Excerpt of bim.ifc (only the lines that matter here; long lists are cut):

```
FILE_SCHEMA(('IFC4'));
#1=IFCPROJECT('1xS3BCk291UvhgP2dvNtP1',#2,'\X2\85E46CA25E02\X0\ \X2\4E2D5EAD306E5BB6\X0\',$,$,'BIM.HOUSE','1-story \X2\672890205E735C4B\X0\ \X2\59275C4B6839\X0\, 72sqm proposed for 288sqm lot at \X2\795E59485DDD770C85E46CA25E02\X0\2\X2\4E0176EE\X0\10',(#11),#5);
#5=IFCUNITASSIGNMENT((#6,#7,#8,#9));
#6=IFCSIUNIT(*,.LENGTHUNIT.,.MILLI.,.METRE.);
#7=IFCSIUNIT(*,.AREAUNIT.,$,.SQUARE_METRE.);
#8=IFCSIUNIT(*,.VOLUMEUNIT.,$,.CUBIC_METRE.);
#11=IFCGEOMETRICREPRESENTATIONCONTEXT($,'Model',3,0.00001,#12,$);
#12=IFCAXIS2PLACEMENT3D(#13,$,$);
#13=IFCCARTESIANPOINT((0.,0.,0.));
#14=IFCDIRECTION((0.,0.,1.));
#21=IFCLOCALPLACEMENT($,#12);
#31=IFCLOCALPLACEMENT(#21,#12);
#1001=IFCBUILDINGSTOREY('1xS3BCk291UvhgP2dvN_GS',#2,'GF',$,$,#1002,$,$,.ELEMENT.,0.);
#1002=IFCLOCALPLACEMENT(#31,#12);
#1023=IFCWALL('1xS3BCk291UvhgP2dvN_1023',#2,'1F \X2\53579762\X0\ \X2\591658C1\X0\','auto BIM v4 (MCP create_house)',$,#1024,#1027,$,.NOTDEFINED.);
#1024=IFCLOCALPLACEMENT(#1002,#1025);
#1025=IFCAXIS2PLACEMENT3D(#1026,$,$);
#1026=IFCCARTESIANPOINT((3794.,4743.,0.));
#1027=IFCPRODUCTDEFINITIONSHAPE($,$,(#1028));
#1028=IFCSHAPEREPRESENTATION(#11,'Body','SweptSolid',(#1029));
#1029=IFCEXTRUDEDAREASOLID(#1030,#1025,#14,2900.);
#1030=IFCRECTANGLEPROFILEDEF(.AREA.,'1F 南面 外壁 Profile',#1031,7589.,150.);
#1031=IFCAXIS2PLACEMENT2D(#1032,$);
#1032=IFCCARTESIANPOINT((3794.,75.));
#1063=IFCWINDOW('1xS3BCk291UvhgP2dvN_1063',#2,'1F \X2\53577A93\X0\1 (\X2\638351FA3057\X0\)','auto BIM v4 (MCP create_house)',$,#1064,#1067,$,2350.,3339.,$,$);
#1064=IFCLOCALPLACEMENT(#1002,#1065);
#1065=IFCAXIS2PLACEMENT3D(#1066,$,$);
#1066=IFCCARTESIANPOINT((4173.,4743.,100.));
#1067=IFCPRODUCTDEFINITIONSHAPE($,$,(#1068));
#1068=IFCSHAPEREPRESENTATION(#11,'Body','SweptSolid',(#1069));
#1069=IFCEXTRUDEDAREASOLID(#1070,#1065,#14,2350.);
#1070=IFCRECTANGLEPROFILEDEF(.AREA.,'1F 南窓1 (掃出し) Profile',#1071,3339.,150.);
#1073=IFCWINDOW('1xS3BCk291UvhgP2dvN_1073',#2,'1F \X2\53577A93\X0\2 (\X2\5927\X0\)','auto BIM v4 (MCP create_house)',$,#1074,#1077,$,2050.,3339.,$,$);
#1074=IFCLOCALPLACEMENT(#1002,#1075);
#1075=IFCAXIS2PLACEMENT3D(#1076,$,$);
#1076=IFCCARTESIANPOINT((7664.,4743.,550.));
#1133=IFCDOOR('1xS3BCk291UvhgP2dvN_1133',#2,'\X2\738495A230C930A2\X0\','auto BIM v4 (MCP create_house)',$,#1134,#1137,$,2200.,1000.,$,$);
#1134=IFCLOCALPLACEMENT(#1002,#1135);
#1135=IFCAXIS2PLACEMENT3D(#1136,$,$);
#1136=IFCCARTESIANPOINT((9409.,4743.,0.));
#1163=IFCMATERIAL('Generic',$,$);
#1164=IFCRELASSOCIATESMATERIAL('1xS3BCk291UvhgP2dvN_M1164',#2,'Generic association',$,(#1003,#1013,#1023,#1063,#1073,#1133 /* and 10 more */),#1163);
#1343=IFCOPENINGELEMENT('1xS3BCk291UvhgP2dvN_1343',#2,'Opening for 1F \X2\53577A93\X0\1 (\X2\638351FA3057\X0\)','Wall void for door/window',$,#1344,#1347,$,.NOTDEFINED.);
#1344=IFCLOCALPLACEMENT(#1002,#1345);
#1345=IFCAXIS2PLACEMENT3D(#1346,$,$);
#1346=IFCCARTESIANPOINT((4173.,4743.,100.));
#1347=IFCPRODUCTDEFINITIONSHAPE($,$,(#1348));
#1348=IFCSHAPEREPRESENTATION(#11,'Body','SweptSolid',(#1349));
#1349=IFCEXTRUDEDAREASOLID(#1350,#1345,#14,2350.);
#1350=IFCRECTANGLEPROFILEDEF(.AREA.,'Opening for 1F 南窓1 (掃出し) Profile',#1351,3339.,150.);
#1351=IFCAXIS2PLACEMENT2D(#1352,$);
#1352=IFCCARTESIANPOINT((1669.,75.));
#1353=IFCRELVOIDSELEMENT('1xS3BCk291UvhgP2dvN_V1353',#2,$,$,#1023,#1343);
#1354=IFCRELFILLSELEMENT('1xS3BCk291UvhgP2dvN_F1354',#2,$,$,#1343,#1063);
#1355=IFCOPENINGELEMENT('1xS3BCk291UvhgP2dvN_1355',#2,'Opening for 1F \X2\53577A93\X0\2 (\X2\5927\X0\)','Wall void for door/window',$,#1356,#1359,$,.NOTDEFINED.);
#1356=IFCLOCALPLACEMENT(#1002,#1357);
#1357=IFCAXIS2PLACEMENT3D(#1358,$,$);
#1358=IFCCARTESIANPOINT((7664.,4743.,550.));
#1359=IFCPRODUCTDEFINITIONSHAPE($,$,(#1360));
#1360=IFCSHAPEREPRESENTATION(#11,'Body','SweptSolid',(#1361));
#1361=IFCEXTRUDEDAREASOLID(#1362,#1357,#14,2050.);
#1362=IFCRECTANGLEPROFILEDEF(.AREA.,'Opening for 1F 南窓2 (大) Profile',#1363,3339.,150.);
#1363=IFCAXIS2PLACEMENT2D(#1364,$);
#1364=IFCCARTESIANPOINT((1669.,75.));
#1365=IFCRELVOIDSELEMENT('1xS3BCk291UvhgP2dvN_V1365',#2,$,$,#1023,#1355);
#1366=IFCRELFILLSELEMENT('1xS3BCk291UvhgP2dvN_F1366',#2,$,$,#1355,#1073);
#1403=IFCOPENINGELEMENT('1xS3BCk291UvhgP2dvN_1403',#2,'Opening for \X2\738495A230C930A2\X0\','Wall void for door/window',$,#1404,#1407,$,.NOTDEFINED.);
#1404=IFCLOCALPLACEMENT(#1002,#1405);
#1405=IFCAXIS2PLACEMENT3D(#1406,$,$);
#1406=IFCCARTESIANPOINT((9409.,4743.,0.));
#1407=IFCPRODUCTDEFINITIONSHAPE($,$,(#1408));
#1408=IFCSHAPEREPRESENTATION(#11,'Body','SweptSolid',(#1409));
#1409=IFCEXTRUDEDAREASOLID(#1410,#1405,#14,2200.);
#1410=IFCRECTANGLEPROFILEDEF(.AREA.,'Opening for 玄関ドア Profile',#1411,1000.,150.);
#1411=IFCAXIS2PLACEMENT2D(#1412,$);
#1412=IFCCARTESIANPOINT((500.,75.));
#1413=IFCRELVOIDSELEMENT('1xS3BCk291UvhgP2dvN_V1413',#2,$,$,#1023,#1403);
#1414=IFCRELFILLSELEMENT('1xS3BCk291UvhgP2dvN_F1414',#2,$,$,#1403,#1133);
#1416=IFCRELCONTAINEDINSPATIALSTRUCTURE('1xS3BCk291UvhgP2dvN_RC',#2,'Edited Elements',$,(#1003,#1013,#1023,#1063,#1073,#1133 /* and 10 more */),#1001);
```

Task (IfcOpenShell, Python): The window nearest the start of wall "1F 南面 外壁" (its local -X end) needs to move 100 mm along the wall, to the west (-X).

```python
import ifcopenshell
import ifcopenshell.api.geometry
import ifcopenshell.util.placement
import ifcopenshell.util.unit

model = ifcopenshell.open("bim.ifc")
unit_scale = ifcopenshell.util.unit.calculate_unit_scale(model)

window = model.by_guid("1xS3BCk291UvhgP2dvN_1063")
opening = window.FillsVoids[0].RelatingOpeningElement
wall = opening.VoidsElements[0].RelatingBuildingElement

wall_matrix = ifcopenshell.util.placement.get_local_placement(wall.ObjectPlacement)
shift = wall_matrix[:3, 0] * -0.1 / unit_scale
before = ifcopenshell.util.placement.get_local_placement(window.ObjectPlacement)[:3, 3].copy()

# The window is not placed relative to its opening, so move both.
for product in (opening, window):
    matrix = ifcopenshell.util.placement.get_local_placement(product.ObjectPlacement)
    matrix[:3, 3] += shift
    ifcopenshell.api.geometry.edit_object_placement(model, product=product, matrix=matrix, is_si=False)

after = ifcopenshell.util.placement.get_local_placement(window.ObjectPlacement)[:3, 3]
print("window moved by", (after - before).round(3) + 0.0)

model.write("bim_v2.ifc")
```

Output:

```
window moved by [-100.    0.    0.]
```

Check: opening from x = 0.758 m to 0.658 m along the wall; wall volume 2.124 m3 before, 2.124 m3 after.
